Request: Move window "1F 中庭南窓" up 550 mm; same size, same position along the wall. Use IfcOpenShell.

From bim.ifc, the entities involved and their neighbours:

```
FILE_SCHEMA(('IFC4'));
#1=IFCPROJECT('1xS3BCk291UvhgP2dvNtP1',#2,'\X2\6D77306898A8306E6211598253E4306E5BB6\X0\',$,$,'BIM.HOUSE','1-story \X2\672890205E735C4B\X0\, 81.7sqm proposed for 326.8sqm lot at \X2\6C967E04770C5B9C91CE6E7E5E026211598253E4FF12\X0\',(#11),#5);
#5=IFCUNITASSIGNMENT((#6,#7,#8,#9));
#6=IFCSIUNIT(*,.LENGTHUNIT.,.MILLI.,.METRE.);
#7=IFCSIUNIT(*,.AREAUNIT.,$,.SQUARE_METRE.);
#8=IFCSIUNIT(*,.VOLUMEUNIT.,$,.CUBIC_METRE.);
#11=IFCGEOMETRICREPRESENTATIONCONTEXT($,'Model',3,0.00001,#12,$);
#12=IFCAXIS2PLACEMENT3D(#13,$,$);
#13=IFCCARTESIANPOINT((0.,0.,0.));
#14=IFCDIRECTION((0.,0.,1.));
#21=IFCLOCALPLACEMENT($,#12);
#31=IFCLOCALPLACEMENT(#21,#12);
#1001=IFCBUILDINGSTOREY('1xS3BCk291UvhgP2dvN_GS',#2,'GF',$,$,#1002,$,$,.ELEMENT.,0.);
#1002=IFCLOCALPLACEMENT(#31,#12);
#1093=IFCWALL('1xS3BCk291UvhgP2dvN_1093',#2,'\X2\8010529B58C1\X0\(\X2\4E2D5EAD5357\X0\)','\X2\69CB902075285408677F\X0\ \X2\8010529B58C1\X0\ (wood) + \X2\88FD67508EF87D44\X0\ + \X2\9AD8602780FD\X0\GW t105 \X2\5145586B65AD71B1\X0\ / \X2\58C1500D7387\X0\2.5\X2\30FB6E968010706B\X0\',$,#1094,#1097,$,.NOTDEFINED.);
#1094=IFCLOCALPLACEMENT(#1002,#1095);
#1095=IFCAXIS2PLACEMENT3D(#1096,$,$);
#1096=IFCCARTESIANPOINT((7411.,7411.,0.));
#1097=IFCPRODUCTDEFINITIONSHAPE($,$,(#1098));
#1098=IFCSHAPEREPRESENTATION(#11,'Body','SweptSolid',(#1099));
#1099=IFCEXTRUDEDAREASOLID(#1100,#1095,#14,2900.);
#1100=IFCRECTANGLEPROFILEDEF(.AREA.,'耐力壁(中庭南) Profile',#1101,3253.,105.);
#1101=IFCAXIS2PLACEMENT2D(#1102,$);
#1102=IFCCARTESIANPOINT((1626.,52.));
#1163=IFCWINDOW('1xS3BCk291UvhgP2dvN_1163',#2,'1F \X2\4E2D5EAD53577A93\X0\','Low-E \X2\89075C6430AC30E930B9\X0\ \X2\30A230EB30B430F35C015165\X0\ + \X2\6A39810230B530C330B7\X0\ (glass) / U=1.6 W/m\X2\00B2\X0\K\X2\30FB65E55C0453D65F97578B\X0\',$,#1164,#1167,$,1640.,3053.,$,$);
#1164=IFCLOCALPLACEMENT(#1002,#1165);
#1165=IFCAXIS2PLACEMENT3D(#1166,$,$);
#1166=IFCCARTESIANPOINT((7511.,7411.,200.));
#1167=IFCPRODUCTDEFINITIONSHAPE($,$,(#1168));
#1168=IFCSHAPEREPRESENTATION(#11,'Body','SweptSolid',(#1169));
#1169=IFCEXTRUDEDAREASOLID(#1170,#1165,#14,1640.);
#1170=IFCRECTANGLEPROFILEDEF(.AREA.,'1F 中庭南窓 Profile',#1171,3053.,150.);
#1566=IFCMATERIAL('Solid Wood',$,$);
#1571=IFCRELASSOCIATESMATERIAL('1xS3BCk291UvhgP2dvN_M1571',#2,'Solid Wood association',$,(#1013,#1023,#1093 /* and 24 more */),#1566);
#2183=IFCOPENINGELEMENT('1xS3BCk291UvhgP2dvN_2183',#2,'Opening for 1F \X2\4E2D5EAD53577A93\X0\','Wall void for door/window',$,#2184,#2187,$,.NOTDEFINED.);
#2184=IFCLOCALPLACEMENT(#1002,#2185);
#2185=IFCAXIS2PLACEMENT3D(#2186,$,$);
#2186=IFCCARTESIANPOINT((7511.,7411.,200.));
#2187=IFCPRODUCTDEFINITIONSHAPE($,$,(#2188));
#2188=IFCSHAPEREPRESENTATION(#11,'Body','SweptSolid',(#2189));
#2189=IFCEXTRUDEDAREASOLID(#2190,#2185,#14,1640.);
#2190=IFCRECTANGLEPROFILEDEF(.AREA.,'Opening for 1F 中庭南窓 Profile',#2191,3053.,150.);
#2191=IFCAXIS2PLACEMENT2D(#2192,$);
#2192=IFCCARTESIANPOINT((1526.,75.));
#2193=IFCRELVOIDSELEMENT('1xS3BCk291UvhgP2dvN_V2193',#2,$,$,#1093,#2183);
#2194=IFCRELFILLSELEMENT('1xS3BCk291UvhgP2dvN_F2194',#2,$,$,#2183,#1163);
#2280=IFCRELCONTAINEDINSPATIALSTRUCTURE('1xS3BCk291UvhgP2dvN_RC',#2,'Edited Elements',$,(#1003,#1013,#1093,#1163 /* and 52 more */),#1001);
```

```python
import numpy as np
import ifcopenshell
import ifcopenshell.api.geometry
import ifcopenshell.util.placement
import ifcopenshell.util.unit

model = ifcopenshell.open("bim.ifc")
unit_scale = ifcopenshell.util.unit.calculate_unit_scale(model)

window = model.by_guid("1xS3BCk291UvhgP2dvN_1163")
opening = window.FillsVoids[0].RelatingOpeningElement
dz = 550.0

shift = np.array([0.0, 0.0, dz])
# The window is not placed relative to its opening, so move both.
for product in (opening, window):
    matrix = ifcopenshell.util.placement.get_local_placement(product.ObjectPlacement)
    matrix[:3, 3] += shift
    ifcopenshell.api.geometry.edit_object_placement(model, product=product, matrix=matrix, is_si=False)

print(f"moved by {dz * unit_scale:+.3f} m")

model.write("bim-out.ifc")
```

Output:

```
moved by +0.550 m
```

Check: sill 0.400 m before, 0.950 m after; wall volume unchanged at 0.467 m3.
